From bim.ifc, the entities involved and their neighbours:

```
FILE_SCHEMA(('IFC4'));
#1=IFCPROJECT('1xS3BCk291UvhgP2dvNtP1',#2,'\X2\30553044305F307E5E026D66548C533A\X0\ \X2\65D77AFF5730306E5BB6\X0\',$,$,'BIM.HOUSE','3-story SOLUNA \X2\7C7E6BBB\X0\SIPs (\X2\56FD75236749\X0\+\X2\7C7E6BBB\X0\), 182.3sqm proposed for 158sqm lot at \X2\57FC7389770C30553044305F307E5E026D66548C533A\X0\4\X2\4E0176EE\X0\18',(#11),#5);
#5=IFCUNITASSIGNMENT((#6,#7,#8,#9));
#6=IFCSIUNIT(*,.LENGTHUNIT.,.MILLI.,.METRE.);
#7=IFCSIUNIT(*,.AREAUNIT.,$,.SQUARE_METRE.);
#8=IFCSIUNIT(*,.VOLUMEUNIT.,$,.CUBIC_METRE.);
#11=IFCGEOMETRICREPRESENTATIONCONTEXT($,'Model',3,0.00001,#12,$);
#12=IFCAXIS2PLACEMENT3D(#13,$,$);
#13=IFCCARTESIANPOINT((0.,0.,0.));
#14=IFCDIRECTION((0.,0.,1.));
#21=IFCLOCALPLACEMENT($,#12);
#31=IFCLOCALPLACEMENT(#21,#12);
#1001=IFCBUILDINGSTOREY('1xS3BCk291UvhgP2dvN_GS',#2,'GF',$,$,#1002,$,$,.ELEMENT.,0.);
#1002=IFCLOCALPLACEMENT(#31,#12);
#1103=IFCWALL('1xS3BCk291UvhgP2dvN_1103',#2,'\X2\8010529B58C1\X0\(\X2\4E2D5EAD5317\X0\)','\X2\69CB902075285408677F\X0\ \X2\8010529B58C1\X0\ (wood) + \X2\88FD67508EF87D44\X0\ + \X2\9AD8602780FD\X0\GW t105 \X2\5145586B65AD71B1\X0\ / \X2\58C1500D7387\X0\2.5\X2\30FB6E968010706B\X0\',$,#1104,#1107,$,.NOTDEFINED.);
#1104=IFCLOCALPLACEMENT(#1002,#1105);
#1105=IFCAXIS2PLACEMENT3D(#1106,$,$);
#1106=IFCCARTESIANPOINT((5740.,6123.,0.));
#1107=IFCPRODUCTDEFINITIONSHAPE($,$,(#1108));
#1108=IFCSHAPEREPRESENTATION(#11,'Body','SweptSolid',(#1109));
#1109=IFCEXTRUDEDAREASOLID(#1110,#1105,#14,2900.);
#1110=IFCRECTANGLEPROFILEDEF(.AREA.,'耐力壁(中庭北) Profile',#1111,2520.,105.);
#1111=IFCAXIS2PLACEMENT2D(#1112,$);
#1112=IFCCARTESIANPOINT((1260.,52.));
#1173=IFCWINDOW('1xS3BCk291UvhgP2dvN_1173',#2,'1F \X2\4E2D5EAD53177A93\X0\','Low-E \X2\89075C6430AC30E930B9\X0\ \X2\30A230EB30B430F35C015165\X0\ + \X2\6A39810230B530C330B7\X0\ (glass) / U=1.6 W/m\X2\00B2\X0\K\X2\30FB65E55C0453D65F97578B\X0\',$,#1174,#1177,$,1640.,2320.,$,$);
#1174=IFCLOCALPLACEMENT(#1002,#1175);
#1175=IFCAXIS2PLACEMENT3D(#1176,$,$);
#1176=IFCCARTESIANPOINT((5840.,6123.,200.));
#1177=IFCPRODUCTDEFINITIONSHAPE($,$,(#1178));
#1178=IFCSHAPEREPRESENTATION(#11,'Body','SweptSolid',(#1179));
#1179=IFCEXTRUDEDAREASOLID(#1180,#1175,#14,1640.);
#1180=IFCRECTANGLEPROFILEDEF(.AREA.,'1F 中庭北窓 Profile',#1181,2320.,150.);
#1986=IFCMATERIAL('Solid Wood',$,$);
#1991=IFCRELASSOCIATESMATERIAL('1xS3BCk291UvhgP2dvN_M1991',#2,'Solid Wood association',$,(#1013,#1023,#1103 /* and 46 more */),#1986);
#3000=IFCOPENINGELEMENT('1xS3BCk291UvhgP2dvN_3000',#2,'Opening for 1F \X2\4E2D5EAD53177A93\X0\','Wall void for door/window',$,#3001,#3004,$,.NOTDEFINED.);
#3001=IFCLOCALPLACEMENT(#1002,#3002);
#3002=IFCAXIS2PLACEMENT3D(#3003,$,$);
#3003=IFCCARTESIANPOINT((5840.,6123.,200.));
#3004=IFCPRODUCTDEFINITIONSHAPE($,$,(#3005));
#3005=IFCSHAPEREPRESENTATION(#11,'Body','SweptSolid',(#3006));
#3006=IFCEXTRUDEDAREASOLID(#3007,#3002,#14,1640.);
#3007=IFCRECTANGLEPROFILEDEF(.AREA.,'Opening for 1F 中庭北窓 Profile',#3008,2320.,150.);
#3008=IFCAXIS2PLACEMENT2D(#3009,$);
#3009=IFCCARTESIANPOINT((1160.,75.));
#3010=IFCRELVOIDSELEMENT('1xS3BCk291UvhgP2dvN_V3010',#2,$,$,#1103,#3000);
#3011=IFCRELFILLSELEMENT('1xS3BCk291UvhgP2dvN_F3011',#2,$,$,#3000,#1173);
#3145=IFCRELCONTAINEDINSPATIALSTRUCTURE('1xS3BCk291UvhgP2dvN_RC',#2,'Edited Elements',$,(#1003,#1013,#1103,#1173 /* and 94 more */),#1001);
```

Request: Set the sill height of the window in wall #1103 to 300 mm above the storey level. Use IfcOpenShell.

```python
import numpy as np
import ifcopenshell
import ifcopenshell.api.geometry
import ifcopenshell.geom
import ifcopenshell.util.element
import ifcopenshell.util.placement
import ifcopenshell.util.shape
import ifcopenshell.util.unit

model = ifcopenshell.open("bim.ifc")
unit_scale = ifcopenshell.util.unit.calculate_unit_scale(model)

window = model.by_id(1173)
opening = window.FillsVoids[0].RelatingOpeningElement
storey = ifcopenshell.util.element.get_container(window, ifc_class="IfcBuildingStorey")
level = ifcopenshell.util.placement.get_local_placement(storey.ObjectPlacement)[2, 3]

# The opening's origin need not be at the sill, so measure its lowest point.
shape = ifcopenshell.geom.create_shape(ifcopenshell.geom.settings(), opening)
bottom = ifcopenshell.util.shape.get_shape_bottom_elevation(shape, shape.geometry) / unit_scale
dz = level + 300.0 - bottom

shift = np.array([0.0, 0.0, dz])
# The window is not placed relative to its opening, so move both.
for product in (opening, window):
    matrix = ifcopenshell.util.placement.get_local_placement(product.ObjectPlacement)
    matrix[:3, 3] += shift
    ifcopenshell.api.geometry.edit_object_placement(model, product=product, matrix=matrix, is_si=False)

print(f"moved by {dz * unit_scale:+.3f} m")

model.write("bim_edited.ifc")
```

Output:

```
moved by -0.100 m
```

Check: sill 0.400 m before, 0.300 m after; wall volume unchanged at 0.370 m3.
